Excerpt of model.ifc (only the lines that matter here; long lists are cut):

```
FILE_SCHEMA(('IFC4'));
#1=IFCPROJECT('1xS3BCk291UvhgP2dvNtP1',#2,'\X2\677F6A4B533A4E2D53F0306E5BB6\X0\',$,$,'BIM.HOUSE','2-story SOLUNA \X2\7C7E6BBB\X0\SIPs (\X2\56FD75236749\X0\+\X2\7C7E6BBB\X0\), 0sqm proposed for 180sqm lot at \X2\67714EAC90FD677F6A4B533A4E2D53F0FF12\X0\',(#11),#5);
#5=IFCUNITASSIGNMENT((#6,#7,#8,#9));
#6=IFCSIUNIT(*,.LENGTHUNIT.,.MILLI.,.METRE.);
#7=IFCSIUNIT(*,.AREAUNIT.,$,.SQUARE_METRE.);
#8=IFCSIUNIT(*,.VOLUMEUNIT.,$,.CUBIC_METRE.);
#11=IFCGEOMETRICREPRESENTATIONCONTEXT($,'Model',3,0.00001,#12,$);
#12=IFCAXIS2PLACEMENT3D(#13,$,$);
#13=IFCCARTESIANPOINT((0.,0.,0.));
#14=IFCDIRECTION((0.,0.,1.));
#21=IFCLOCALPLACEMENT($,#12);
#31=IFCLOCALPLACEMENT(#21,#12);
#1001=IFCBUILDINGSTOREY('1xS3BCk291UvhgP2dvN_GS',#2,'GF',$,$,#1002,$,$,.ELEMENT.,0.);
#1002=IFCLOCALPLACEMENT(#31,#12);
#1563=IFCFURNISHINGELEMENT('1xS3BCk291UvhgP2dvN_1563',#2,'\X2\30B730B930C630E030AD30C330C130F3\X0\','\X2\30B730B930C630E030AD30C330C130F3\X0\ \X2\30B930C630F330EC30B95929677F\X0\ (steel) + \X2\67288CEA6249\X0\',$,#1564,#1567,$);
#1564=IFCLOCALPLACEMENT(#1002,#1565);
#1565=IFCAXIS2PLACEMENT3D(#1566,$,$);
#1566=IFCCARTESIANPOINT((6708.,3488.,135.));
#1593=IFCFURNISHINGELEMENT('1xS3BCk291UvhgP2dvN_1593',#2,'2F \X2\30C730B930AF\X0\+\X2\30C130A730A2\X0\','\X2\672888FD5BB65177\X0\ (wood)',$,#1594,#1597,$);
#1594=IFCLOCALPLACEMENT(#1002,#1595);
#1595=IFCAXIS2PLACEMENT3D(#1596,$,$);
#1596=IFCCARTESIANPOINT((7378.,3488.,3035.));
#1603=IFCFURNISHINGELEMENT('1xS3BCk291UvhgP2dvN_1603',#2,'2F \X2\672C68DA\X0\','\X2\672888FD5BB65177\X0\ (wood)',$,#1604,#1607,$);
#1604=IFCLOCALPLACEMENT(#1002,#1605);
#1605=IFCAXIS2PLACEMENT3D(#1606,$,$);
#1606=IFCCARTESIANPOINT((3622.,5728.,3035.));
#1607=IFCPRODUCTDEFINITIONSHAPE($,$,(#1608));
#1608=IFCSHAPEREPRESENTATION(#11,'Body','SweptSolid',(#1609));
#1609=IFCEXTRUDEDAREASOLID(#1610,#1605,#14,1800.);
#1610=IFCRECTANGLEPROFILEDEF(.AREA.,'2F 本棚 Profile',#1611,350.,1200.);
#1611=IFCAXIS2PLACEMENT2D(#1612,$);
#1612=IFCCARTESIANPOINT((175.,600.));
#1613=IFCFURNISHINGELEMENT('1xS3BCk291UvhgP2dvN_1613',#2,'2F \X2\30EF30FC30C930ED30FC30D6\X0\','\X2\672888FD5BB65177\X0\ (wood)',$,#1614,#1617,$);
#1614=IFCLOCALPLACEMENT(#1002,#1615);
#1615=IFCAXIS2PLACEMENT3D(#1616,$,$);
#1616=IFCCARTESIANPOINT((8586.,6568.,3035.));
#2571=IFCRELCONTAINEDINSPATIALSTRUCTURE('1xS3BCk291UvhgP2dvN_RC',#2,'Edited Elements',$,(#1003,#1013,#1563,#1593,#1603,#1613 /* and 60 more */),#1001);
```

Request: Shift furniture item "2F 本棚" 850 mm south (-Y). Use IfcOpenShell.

```python
import ifcopenshell
import ifcopenshell.api.geometry
import ifcopenshell.util.placement
import ifcopenshell.util.unit

model = ifcopenshell.open("model.ifc")
unit_scale = ifcopenshell.util.unit.calculate_unit_scale(model)

item = model.by_guid("1xS3BCk291UvhgP2dvN_1603")
matrix = ifcopenshell.util.placement.get_local_placement(item.ObjectPlacement)
matrix[1, 3] -= 0.85 / unit_scale
ifcopenshell.api.geometry.edit_object_placement(model, product=item, matrix=matrix, is_si=False)

print(ifcopenshell.util.placement.get_local_placement(item.ObjectPlacement).round(3) + 0.0)

model.write("model_rev.ifc")
```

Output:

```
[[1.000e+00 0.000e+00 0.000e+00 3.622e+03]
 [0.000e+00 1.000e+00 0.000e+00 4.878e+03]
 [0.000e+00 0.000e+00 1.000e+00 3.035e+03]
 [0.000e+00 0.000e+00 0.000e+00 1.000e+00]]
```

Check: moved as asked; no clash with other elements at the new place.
